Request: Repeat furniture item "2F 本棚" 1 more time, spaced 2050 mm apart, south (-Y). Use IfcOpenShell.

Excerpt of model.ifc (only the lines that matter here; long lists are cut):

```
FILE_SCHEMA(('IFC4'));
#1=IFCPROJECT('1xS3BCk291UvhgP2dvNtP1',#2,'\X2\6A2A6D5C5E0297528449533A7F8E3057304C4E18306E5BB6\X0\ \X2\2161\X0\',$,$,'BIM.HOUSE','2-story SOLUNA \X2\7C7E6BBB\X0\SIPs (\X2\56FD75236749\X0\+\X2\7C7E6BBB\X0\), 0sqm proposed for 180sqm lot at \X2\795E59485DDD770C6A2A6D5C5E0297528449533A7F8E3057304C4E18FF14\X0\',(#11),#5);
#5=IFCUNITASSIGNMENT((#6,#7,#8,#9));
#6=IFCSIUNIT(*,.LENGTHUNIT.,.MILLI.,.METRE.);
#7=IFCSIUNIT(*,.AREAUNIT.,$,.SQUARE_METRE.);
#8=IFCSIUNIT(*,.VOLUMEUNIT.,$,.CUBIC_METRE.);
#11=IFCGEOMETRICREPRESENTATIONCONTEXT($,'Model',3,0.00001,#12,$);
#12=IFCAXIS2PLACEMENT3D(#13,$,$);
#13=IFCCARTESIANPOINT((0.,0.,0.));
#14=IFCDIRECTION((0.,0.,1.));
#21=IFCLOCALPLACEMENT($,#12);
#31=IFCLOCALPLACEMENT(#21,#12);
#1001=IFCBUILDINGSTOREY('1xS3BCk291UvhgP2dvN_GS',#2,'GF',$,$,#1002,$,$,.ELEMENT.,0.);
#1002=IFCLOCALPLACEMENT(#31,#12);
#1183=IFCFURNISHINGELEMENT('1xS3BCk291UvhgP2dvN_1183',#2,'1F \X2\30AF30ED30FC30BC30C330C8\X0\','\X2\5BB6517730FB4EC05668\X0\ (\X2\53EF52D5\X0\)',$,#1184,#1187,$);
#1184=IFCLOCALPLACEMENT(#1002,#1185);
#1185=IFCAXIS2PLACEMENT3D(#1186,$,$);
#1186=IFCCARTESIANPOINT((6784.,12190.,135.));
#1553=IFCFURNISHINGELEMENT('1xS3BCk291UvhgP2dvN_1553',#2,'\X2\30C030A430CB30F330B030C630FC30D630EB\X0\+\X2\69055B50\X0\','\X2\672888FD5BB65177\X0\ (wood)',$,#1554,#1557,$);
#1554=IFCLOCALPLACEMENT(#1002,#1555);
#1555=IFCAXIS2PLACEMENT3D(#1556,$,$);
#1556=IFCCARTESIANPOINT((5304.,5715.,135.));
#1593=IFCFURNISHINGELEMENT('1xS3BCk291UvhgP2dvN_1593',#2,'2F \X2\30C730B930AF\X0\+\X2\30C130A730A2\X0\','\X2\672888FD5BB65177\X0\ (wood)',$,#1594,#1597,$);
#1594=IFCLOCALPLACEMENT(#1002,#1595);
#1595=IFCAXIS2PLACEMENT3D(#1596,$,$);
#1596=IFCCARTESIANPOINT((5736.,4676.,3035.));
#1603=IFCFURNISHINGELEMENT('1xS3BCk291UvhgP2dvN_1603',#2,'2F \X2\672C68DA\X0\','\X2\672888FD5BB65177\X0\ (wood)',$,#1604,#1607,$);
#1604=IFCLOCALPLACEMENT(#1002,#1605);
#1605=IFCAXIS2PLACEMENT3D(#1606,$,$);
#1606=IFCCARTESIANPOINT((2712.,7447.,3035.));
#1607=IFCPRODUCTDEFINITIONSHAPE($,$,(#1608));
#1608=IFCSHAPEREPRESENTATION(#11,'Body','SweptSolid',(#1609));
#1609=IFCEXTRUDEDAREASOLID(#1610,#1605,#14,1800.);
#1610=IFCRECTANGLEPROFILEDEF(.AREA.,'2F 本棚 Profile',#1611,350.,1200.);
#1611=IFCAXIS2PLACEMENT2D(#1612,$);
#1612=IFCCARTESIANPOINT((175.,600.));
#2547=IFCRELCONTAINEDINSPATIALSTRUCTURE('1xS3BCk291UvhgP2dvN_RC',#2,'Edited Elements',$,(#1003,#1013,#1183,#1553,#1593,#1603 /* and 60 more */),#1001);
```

```python
import numpy as np
import ifcopenshell
import ifcopenshell.api.geometry
import ifcopenshell.api.root
import ifcopenshell.util.element
import ifcopenshell.util.placement
import ifcopenshell.util.unit

model = ifcopenshell.open("model.ifc")
unit_scale = ifcopenshell.util.unit.calculate_unit_scale(model)


def reuse_history(source, copy):
    """copy_class also copies each property set's owner history, people and application; keep the originals."""
    for rel in copy.IsDefinedBy:
        if rel.is_a("IfcRelDefinesByProperties") and (history := rel.RelatingPropertyDefinition.OwnerHistory):
            rel.RelatingPropertyDefinition.OwnerHistory = source.OwnerHistory
            ifcopenshell.util.element.remove_deep2(model, history)


source = model.by_guid("1xS3BCk291UvhgP2dvN_1603")
base = ifcopenshell.util.placement.get_local_placement(source.ObjectPlacement)
step = np.array([0.0, -1.0, 0.0]) * 2.05 / unit_scale

for i in range(1, 2):
    copy = ifcopenshell.api.root.copy_class(model, product=source)
    copy.Representation = ifcopenshell.util.element.copy_deep(
        model, source.Representation, exclude=["IfcGeometricRepresentationContext", "IfcRepresentationMap"]
    )
    reuse_history(source, copy)
    matrix = base.copy()
    matrix[:3, 3] += i * step
    print("added at", matrix[:3, 3].round(3) + 0.0)
    ifcopenshell.api.geometry.edit_object_placement(model, product=copy, matrix=matrix, is_si=False)

model.write("model_edited.ifc")
```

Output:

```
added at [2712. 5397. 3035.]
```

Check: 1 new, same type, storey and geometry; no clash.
